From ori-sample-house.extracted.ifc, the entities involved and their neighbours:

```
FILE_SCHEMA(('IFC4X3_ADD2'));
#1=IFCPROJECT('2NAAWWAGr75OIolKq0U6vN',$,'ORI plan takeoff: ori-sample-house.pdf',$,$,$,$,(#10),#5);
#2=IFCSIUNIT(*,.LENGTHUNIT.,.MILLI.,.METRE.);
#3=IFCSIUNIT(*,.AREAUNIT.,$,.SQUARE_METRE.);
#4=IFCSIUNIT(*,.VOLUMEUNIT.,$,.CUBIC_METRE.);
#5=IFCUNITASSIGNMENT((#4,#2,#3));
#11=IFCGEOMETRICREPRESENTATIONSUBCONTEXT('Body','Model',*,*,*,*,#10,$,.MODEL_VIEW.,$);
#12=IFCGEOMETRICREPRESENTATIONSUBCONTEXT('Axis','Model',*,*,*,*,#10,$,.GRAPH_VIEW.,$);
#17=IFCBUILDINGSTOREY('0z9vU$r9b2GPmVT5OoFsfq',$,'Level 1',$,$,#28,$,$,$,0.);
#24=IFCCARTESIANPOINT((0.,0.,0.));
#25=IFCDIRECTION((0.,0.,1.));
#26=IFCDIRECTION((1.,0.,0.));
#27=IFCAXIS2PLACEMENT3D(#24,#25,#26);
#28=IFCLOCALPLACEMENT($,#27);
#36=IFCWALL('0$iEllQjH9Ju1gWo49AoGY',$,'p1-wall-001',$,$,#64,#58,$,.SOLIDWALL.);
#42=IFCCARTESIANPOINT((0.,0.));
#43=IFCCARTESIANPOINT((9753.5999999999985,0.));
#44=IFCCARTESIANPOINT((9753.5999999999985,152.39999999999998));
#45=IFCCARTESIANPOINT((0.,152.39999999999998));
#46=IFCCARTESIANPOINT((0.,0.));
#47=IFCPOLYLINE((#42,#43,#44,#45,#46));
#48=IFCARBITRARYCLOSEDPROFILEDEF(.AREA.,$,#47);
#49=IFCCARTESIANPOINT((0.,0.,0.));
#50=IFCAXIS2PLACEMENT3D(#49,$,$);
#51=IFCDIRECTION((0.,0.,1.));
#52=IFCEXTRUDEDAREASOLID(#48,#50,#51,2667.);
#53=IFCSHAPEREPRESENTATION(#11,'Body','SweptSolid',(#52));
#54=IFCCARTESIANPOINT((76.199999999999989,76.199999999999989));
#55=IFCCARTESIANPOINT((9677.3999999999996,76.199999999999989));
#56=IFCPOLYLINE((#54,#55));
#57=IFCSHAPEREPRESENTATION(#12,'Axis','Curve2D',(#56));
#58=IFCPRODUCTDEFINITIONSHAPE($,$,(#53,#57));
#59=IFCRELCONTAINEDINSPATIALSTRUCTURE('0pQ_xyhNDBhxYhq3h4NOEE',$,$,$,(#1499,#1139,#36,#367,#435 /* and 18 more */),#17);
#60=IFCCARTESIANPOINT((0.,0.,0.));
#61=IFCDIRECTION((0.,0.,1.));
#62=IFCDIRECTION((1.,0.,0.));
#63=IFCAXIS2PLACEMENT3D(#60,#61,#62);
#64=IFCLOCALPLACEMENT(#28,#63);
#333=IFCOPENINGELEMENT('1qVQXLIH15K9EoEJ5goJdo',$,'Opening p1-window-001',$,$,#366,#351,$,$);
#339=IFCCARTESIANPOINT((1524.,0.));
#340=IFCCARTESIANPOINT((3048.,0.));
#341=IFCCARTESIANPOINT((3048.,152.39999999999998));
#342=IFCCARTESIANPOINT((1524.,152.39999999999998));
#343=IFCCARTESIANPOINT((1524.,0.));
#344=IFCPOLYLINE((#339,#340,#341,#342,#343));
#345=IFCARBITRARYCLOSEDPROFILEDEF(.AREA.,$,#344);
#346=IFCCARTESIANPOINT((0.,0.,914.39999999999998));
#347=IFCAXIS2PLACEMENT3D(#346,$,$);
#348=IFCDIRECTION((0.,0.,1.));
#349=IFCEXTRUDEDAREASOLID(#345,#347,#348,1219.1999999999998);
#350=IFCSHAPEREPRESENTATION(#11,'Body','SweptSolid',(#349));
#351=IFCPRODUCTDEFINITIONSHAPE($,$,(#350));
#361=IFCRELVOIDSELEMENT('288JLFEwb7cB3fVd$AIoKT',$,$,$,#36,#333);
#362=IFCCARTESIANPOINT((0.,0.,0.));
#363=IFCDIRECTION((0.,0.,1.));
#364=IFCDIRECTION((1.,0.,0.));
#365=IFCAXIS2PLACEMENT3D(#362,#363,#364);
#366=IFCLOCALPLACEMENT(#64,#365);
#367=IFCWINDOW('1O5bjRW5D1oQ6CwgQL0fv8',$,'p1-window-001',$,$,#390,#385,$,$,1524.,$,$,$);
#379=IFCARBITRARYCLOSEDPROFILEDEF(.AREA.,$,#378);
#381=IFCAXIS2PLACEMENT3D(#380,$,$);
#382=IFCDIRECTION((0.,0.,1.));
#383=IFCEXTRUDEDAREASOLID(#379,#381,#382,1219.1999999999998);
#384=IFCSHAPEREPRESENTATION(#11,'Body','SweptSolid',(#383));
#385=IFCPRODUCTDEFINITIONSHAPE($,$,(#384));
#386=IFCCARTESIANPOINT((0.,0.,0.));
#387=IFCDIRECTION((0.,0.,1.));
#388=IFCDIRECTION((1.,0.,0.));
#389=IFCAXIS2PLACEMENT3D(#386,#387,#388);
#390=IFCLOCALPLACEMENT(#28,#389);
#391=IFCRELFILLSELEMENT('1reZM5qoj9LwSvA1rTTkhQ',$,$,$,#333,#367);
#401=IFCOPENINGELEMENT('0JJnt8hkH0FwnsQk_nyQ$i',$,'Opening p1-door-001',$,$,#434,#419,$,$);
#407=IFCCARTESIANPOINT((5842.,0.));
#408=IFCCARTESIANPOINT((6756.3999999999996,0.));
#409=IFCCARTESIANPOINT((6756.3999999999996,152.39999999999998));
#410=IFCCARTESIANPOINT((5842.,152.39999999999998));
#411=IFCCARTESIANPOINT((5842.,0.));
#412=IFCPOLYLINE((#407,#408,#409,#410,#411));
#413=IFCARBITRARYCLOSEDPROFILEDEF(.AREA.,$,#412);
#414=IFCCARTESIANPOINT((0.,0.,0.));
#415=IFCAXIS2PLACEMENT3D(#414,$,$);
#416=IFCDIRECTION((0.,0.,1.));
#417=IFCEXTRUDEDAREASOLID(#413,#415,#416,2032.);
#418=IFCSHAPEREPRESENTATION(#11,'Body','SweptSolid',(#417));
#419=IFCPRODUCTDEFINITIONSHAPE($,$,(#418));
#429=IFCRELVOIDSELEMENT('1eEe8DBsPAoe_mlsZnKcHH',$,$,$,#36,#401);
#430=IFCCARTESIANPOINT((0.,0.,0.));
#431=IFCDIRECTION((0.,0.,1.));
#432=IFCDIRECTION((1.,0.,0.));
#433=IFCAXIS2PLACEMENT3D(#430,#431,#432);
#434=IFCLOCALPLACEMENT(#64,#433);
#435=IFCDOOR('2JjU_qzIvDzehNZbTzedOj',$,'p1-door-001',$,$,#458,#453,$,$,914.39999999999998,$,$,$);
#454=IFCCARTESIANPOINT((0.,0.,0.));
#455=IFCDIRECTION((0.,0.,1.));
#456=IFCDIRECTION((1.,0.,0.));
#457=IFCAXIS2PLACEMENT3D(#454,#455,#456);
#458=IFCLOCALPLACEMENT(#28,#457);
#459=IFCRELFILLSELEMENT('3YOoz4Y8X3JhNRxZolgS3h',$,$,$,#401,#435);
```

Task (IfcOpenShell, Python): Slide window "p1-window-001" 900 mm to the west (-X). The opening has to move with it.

```python
import ifcopenshell
import ifcopenshell.api.geometry
import ifcopenshell.util.placement
import ifcopenshell.util.unit

model = ifcopenshell.open("ori-sample-house.extracted.ifc")
unit_scale = ifcopenshell.util.unit.calculate_unit_scale(model)

window = model.by_guid("1O5bjRW5D1oQ6CwgQL0fv8")
opening = window.FillsVoids[0].RelatingOpeningElement
wall = opening.VoidsElements[0].RelatingBuildingElement

wall_matrix = ifcopenshell.util.placement.get_local_placement(wall.ObjectPlacement)
shift = wall_matrix[:3, 0] * -0.9 / unit_scale
before = ifcopenshell.util.placement.get_local_placement(window.ObjectPlacement)[:3, 3].copy()

# The window is not placed relative to its opening, so move both.
for product in (opening, window):
    matrix = ifcopenshell.util.placement.get_local_placement(product.ObjectPlacement)
    matrix[:3, 3] += shift
    ifcopenshell.api.geometry.edit_object_placement(model, product=product, matrix=matrix, is_si=False)

after = ifcopenshell.util.placement.get_local_placement(window.ObjectPlacement)[:3, 3]
print("window moved by", (after - before).round(3) + 0.0)

model.write("ori-sample-house.extracted-out.ifc")
```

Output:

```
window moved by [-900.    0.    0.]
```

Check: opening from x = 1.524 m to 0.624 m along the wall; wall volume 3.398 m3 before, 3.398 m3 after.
